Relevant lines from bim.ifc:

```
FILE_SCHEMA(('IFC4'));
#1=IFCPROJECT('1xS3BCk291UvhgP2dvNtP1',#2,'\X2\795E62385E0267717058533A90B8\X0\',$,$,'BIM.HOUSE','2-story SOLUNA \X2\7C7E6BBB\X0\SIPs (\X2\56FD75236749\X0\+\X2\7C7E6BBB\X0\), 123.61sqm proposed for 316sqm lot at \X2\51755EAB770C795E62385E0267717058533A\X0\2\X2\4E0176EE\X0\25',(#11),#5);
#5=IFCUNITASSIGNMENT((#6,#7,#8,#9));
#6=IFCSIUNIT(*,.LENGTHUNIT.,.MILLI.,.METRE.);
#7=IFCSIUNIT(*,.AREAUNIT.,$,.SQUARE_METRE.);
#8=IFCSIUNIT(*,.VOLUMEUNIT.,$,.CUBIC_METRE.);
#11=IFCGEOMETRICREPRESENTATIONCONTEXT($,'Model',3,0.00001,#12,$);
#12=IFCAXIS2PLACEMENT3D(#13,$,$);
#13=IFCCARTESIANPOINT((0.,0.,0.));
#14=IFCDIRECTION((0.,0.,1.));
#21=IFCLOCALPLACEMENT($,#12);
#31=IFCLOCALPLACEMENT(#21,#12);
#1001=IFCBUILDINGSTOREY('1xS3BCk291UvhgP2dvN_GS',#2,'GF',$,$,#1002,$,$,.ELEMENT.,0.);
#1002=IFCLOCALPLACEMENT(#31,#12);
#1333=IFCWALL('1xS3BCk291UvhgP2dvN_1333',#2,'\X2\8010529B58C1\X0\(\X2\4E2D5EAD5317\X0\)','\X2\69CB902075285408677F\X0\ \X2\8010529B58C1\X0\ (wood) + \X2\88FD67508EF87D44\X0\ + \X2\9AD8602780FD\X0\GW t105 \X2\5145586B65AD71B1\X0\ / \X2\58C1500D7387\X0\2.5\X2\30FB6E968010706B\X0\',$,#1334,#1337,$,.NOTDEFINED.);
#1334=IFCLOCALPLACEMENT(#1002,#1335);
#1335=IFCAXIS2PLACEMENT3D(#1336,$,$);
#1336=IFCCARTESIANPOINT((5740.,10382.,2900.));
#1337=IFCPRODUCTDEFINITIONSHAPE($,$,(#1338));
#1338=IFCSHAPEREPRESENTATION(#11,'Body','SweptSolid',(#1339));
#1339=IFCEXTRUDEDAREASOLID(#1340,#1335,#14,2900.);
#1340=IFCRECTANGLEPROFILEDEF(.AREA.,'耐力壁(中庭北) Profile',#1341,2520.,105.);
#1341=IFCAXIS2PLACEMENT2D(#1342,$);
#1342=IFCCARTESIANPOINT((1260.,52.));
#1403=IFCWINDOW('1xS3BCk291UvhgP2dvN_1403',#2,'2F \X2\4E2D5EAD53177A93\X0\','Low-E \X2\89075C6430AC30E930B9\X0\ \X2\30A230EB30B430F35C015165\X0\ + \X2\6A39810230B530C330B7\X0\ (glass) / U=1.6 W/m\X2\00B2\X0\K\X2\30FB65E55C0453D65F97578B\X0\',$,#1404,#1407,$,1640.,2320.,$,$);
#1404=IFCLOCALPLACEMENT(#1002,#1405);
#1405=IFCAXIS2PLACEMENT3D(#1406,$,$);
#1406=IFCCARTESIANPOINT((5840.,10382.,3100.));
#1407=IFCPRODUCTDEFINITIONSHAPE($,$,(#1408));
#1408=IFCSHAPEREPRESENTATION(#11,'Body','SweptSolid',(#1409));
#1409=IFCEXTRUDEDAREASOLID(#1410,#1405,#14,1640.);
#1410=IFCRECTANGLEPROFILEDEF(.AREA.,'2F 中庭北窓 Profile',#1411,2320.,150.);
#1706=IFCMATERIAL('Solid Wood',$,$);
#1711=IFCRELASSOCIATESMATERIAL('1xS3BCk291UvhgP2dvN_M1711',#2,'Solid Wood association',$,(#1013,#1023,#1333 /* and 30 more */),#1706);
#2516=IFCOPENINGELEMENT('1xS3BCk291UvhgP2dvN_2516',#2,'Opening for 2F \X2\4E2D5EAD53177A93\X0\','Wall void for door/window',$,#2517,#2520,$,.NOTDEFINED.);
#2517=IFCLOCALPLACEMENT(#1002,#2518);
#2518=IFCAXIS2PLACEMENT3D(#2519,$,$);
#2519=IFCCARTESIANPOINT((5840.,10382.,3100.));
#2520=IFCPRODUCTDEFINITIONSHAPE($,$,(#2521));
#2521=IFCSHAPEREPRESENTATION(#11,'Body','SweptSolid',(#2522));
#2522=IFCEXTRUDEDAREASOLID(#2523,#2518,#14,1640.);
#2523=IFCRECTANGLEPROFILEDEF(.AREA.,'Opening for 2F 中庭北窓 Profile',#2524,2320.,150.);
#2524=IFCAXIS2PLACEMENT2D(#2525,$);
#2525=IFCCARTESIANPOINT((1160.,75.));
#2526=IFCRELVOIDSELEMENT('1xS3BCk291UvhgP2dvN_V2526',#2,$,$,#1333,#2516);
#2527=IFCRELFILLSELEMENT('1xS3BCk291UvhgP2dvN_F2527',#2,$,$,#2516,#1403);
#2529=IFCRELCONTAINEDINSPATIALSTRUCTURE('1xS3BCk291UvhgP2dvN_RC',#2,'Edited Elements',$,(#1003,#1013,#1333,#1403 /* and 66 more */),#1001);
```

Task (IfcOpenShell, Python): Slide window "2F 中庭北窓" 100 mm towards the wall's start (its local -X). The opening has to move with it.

```python
import ifcopenshell
import ifcopenshell.api.geometry
import ifcopenshell.util.placement

model = ifcopenshell.open("bim.ifc")

window = model.by_id(1403)
opening = window.FillsVoids[0].RelatingOpeningElement
wall = opening.VoidsElements[0].RelatingBuildingElement

wall_matrix = ifcopenshell.util.placement.get_local_placement(wall.ObjectPlacement)
shift = wall_matrix[:3, 0] * -100.0
before = ifcopenshell.util.placement.get_local_placement(window.ObjectPlacement)[:3, 3].copy()

# The window is not placed relative to its opening, so move both.
for product in (opening, window):
    matrix = ifcopenshell.util.placement.get_local_placement(product.ObjectPlacement)
    matrix[:3, 3] += shift
    ifcopenshell.api.geometry.edit_object_placement(model, product=product, matrix=matrix, is_si=False)

after = ifcopenshell.util.placement.get_local_placement(window.ObjectPlacement)[:3, 3]
print("window moved by", (after - before).round(3) + 0.0)

model.write("bim_edited.ifc")
```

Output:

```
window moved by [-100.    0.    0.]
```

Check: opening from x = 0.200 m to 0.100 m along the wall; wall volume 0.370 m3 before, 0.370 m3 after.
